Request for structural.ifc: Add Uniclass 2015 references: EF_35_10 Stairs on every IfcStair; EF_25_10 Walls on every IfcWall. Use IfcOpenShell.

First a look at what the model holds.

```python
import ifcopenshell

model = ifcopenshell.open("structural.ifc")
print(model.schema)
print("classifications:", [c.Name for c in model.by_type("IfcClassification")])
for ifc_class in ("IfcDoor", "IfcRoof", "IfcStair", "IfcWall", "IfcWindow"):
    print(ifc_class, len(model.by_type(ifc_class)))
```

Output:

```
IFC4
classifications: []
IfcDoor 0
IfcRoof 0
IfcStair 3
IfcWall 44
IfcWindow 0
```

```python
import ifcopenshell
import ifcopenshell.api.classification

model = ifcopenshell.open("structural.ifc")

system = ifcopenshell.api.classification.add_classification(model, classification="Uniclass 2015")

codes = {
    "IfcStair": ("EF_35_10", "Stairs"),
    "IfcWall": ("EF_25_10", "Walls"),
}
for ifc_class, (code, name) in codes.items():
    products = model.by_type(ifc_class)
    ifcopenshell.api.classification.add_reference(
        model, products=products, classification=system, identification=code, name=name
    )
    print(code, len(products))

model.write("structural-out.ifc")
```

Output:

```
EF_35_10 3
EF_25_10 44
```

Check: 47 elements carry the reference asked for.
